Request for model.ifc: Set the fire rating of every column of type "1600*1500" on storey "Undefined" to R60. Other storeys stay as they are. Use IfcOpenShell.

First a look at what the model holds.

```python
import ifcopenshell
import ifcopenshell.util.element

model = ifcopenshell.open("model.ifc")
print(model.schema)
storey = next(s for s in model.by_type("IfcBuildingStorey") if s.Name == "Undefined")
columns = [e for e in ifcopenshell.util.element.get_decomposition(storey) if e.is_a("IfcColumn")]
seen = {}
for e in columns:
    element_type = ifcopenshell.util.element.get_type(e)
    key = (element_type.Name if element_type != e and element_type else None, ifcopenshell.util.element.get_pset(e, "Pset_ColumnCommon", "FireRating"))
    seen[key] = seen.get(key, 0) + 1
for (name, value), count in sorted(seen.items(), key=str):
    print(count, "x", name, "|", value)
```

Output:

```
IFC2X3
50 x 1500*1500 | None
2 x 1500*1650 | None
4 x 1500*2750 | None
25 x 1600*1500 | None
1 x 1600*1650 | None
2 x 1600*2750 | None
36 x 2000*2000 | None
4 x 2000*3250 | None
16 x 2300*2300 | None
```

```python
import ifcopenshell
import ifcopenshell.api.pset
import ifcopenshell.util.element

model = ifcopenshell.open("model.ifc")

storey = next(s for s in model.by_type("IfcBuildingStorey") if s.Name == "Undefined")
columns = [e for e in ifcopenshell.util.element.get_decomposition(storey) if e.is_a("IfcColumn")]

count = 0
for e in columns:
    element_type = ifcopenshell.util.element.get_type(e)
    if element_type in (None, e) or element_type.Name != "1600*1500":
        continue
    found = ifcopenshell.util.element.get_pset(e, "Pset_ColumnCommon", should_inherit=False)
    if found:
        pset = model.by_id(found["id"])
        if len(ifcopenshell.util.element.get_elements_by_pset(pset)) > 1:
            pset = ifcopenshell.api.pset.unshare_pset(model, products=[e], pset=pset)[0]
    else:
        pset = ifcopenshell.api.pset.add_pset(model, product=e, name="Pset_ColumnCommon")
    ifcopenshell.api.pset.edit_pset(model, pset=pset, properties={"FireRating": "R60"})
    count += 1

print(count, "columns updated")

model.write("model_edited.ifc")
```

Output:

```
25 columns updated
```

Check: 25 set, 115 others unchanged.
